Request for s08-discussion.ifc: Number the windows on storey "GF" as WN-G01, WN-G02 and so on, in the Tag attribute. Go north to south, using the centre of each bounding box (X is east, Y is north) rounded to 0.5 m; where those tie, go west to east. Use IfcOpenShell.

First a look at what the model holds.

```python
import ifcopenshell
import ifcopenshell.util.element
import ifcopenshell.util.placement

model = ifcopenshell.open("s08-discussion.ifc")
print(model.schema)
storey = next(s for s in model.by_type("IfcBuildingStorey") if s.Name == "GF")
windows = [e for e in ifcopenshell.util.element.get_decomposition(storey) if e.is_a("IfcWindow")]
for e in sorted(windows, key=lambda e: e.id()):
    origin = ifcopenshell.util.placement.get_local_placement(e.ObjectPlacement)[:3, 3]
    print(e.id(), e.Tag, e.Name, origin.round(2) + 0.0, sep=" | ")
```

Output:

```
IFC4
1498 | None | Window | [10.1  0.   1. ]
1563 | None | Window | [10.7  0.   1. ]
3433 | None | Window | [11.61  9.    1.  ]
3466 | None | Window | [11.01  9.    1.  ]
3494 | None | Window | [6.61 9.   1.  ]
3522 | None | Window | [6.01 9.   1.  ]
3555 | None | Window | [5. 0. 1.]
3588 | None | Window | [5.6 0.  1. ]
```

```python
import ifcopenshell
import ifcopenshell.geom
import ifcopenshell.util.element
import ifcopenshell.util.shape

model = ifcopenshell.open("s08-discussion.ifc")
settings = ifcopenshell.geom.settings()
settings.set("use-world-coords", True)


def centre(element):
    shape = ifcopenshell.geom.create_shape(settings, element)
    return ifcopenshell.util.shape.get_bbox_centroid(shape.geometry)


storey = next(s for s in model.by_type("IfcBuildingStorey") if s.Name == "GF")
windows = [e for e in ifcopenshell.util.element.get_decomposition(storey) if e.is_a("IfcWindow")]

# Insertion points can sit at a corner or the storey origin, so sort by the geometry (in metres).
centres = {e: centre(e) for e in windows}
windows.sort(key=lambda e: (-round(centres[e][1] / 0.5), centres[e][0]))

for i, e in enumerate(windows, start=1):
    number = f"WN-G{i:02d}"
    e.Tag = number
    print(e.id(), number)

model.write("s08-discussion_rev.ifc")
```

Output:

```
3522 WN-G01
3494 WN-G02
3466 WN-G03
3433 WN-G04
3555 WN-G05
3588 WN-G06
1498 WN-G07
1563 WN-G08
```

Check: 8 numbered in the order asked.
